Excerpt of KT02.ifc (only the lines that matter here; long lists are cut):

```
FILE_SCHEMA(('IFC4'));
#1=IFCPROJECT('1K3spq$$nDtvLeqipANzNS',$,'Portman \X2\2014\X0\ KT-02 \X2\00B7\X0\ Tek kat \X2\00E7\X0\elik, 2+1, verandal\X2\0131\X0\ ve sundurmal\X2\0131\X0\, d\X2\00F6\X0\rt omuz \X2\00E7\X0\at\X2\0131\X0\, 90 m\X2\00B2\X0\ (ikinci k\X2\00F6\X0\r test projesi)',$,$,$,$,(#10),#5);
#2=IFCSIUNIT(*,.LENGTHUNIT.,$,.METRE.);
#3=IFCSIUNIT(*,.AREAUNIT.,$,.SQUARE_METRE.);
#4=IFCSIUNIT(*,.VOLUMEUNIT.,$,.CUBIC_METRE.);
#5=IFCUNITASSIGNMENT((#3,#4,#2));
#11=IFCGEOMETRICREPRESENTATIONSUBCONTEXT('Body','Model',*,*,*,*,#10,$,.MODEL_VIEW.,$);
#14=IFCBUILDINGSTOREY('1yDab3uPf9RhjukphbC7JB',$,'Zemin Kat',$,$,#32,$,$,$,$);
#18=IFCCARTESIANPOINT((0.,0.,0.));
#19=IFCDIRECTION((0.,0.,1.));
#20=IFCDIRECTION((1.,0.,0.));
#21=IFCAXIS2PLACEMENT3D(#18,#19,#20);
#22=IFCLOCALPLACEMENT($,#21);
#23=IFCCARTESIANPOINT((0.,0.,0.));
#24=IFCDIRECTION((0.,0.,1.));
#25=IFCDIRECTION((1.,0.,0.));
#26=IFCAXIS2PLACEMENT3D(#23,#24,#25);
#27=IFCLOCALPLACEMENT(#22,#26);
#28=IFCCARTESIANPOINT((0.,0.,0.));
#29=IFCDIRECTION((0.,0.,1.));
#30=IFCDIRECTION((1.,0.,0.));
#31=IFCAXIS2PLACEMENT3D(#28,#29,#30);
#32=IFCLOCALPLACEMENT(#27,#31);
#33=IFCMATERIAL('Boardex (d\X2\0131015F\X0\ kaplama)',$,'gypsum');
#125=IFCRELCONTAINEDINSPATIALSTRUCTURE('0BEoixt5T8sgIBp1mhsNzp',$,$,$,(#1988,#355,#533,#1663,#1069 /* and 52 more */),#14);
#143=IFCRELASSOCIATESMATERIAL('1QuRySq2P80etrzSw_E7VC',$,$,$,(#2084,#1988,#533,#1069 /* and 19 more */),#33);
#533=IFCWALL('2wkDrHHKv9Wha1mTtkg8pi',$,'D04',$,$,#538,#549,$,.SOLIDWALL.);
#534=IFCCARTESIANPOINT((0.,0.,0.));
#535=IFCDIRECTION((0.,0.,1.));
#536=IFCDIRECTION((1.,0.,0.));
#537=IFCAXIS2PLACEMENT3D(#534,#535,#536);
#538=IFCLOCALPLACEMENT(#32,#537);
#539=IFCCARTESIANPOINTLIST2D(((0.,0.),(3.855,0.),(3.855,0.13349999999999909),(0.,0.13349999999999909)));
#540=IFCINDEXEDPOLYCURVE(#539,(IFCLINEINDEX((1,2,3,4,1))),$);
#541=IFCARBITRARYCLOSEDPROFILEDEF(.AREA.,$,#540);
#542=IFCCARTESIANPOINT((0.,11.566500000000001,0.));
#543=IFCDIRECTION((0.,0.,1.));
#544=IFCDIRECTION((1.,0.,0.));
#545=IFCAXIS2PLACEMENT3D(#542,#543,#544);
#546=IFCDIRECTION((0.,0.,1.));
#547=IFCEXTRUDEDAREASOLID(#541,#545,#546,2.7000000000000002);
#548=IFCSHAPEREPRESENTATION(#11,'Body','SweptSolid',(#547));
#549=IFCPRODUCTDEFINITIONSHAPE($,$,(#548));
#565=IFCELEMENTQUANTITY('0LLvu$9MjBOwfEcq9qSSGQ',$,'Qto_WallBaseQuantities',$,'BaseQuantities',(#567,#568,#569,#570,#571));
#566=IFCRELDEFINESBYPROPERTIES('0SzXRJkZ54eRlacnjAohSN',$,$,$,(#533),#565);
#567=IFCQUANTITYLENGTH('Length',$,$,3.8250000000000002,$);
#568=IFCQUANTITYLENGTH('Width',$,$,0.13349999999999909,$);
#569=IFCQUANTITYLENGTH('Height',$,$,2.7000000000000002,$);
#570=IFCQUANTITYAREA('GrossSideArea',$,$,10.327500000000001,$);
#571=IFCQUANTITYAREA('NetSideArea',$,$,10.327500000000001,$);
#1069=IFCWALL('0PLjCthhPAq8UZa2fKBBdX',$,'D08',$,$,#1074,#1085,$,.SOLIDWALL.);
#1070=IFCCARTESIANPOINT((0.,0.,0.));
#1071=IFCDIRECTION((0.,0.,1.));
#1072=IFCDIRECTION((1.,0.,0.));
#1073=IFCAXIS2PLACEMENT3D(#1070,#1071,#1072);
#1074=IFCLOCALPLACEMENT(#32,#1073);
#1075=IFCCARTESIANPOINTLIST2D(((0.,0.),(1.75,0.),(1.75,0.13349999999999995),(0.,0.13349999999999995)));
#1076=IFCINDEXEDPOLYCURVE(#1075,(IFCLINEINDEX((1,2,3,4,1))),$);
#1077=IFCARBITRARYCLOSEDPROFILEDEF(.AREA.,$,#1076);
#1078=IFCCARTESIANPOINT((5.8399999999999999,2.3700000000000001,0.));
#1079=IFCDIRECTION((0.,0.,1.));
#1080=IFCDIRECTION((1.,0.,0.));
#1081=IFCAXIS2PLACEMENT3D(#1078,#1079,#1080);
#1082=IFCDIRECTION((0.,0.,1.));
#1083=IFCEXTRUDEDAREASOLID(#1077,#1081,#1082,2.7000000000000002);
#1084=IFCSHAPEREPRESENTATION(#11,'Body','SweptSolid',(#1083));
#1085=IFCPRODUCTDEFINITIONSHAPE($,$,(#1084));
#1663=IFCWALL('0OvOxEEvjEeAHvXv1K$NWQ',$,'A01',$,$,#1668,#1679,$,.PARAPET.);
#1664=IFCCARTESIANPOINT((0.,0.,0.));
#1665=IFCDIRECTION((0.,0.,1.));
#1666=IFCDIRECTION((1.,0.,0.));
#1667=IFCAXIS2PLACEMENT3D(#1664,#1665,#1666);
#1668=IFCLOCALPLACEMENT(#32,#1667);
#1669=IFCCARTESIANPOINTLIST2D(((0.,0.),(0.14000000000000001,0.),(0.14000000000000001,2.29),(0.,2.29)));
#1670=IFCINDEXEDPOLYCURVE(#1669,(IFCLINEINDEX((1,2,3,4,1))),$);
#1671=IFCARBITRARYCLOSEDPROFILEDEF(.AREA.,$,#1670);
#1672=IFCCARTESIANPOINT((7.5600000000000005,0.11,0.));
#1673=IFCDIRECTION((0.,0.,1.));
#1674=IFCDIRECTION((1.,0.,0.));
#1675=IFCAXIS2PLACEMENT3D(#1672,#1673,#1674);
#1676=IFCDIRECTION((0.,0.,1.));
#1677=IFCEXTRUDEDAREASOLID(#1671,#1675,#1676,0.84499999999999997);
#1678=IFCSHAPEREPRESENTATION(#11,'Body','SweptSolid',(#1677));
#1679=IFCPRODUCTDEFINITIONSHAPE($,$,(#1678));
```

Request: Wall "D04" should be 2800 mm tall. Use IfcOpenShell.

```python
import ifcopenshell
import ifcopenshell.api.pset
import ifcopenshell.geom
import ifcopenshell.util.element
import ifcopenshell.util.representation
import ifcopenshell.util.shape
import ifcopenshell.util.unit

model = ifcopenshell.open("KT02.ifc")
unit_scale = ifcopenshell.util.unit.calculate_unit_scale(model)
area_scale = ifcopenshell.util.unit.calculate_unit_scale(model, "AREAUNIT")
settings = ifcopenshell.geom.settings()


def volume(element):
    """Net volume in cubic metres, openings subtracted."""
    shape = ifcopenshell.geom.create_shape(settings, element)
    return ifcopenshell.util.shape.get_volume(shape.geometry)


wall = model.by_guid("2wkDrHHKv9Wha1mTtkg8pi")
before = volume(wall)

body = ifcopenshell.util.representation.get_representation(wall, "Model", "Body")
solid = body.Items[0]
old_height = solid.Depth
solid.Depth = 2.8 / unit_scale
after = volume(wall)
thickness = 0.1335  # wall thickness in metres

# Update the stored height, areas and volumes.
qto = model.by_id(ifcopenshell.util.element.get_pset(wall, "Qto_WallBaseQuantities", should_inherit=False)["id"])
ifcopenshell.api.pset.edit_qto(model, qto=qto, properties={
    "Height": solid.Depth,
    "GrossSideArea": ifcopenshell.util.element.get_pset(wall, "Qto_WallBaseQuantities", "GrossSideArea") * solid.Depth / old_height,
    "NetSideArea": after / thickness / area_scale,
})

print(f"height {old_height:g} -> {solid.Depth:g}, volume {before:.3f} -> {after:.3f} m3")

model.write("KT02-out.ifc")
```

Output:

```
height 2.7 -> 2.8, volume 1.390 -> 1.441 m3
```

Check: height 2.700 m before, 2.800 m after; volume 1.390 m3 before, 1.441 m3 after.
